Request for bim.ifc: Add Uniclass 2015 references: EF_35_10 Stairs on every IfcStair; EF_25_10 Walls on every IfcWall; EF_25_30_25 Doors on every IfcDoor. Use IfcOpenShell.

First a look at what the model holds.

```python
import ifcopenshell

model = ifcopenshell.open("bim.ifc")
print(model.schema)
print("classifications:", [c.Name for c in model.by_type("IfcClassification")])
for ifc_class in ("IfcDoor", "IfcRoof", "IfcStair", "IfcWall", "IfcWindow"):
    print(ifc_class, len(model.by_type(ifc_class)))
```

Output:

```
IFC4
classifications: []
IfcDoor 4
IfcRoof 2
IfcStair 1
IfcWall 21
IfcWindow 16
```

```python
import ifcopenshell
import ifcopenshell.api.classification

model = ifcopenshell.open("bim.ifc")

system = ifcopenshell.api.classification.add_classification(model, classification="Uniclass 2015")

codes = {
    "IfcStair": ("EF_35_10", "Stairs"),
    "IfcWall": ("EF_25_10", "Walls"),
    "IfcDoor": ("EF_25_30_25", "Doors"),
}
for ifc_class, (code, name) in codes.items():
    products = model.by_type(ifc_class)
    ifcopenshell.api.classification.add_reference(
        model, products=products, classification=system, identification=code, name=name
    )
    print(code, len(products))

model.write("bim_updated.ifc")
```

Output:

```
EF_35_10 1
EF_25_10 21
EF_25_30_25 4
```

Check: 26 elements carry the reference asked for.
